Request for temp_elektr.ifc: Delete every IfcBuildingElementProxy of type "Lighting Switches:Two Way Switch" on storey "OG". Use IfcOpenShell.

First a look at what the model holds.

```python
import ifcopenshell
import ifcopenshell.util.element

model = ifcopenshell.open("temp_elektr.ifc")
print(model.schema)
storey = next(s for s in model.by_type("IfcBuildingStorey") if s.Name == "OG")
proxies = [e for e in ifcopenshell.util.element.get_decomposition(storey) if e.is_a("IfcBuildingElementProxy")]
seen = {}
for e in proxies:
    element_type = ifcopenshell.util.element.get_type(e)
    name = element_type.Name if element_type not in (None, e) else None
    seen[name] = seen.get(name, 0) + 1
for name, count in sorted(seen.items(), key=str):
    print(count, "x", name)
```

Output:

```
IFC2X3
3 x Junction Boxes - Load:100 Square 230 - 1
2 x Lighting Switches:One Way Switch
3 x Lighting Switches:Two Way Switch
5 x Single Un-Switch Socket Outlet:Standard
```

```python
import ifcopenshell
import ifcopenshell.api.root
import ifcopenshell.util.element

model = ifcopenshell.open("temp_elektr.ifc")

storey = next(s for s in model.by_type("IfcBuildingStorey") if s.Name == "OG")
proxies = [e for e in ifcopenshell.util.element.get_decomposition(storey) if e.is_a("IfcBuildingElementProxy")]
targets = [e for e in proxies if (t := ifcopenshell.util.element.get_type(e)) not in (None, e) and t.Name == "Lighting Switches:Two Way Switch"]

for e in targets:
    ifcopenshell.api.root.remove_product(model, product=e)
print(len(targets), "removed")

model.write("temp_elektr-out.ifc")
```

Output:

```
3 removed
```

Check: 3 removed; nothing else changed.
